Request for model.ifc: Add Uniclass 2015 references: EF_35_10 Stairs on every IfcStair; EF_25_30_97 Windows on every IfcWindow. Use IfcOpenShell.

First a look at what the model holds.

```python
import ifcopenshell

model = ifcopenshell.open("model.ifc")
print(model.schema)
print("classifications:", [c.Name for c in model.by_type("IfcClassification")])
for ifc_class in ("IfcDoor", "IfcRoof", "IfcStair", "IfcWall", "IfcWindow"):
    print(ifc_class, len(model.by_type(ifc_class)))
```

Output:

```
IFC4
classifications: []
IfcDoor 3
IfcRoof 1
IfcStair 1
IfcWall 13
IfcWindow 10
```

```python
import ifcopenshell
import ifcopenshell.api.classification

model = ifcopenshell.open("model.ifc")

system = ifcopenshell.api.classification.add_classification(model, classification="Uniclass 2015")

codes = {
    "IfcStair": ("EF_35_10", "Stairs"),
    "IfcWindow": ("EF_25_30_97", "Windows"),
}
for ifc_class, (code, name) in codes.items():
    products = model.by_type(ifc_class)
    ifcopenshell.api.classification.add_reference(
        model, products=products, classification=system, identification=code, name=name
    )
    print(code, len(products))

model.write("model_edited.ifc")
```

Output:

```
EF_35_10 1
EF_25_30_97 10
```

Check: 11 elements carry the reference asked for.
